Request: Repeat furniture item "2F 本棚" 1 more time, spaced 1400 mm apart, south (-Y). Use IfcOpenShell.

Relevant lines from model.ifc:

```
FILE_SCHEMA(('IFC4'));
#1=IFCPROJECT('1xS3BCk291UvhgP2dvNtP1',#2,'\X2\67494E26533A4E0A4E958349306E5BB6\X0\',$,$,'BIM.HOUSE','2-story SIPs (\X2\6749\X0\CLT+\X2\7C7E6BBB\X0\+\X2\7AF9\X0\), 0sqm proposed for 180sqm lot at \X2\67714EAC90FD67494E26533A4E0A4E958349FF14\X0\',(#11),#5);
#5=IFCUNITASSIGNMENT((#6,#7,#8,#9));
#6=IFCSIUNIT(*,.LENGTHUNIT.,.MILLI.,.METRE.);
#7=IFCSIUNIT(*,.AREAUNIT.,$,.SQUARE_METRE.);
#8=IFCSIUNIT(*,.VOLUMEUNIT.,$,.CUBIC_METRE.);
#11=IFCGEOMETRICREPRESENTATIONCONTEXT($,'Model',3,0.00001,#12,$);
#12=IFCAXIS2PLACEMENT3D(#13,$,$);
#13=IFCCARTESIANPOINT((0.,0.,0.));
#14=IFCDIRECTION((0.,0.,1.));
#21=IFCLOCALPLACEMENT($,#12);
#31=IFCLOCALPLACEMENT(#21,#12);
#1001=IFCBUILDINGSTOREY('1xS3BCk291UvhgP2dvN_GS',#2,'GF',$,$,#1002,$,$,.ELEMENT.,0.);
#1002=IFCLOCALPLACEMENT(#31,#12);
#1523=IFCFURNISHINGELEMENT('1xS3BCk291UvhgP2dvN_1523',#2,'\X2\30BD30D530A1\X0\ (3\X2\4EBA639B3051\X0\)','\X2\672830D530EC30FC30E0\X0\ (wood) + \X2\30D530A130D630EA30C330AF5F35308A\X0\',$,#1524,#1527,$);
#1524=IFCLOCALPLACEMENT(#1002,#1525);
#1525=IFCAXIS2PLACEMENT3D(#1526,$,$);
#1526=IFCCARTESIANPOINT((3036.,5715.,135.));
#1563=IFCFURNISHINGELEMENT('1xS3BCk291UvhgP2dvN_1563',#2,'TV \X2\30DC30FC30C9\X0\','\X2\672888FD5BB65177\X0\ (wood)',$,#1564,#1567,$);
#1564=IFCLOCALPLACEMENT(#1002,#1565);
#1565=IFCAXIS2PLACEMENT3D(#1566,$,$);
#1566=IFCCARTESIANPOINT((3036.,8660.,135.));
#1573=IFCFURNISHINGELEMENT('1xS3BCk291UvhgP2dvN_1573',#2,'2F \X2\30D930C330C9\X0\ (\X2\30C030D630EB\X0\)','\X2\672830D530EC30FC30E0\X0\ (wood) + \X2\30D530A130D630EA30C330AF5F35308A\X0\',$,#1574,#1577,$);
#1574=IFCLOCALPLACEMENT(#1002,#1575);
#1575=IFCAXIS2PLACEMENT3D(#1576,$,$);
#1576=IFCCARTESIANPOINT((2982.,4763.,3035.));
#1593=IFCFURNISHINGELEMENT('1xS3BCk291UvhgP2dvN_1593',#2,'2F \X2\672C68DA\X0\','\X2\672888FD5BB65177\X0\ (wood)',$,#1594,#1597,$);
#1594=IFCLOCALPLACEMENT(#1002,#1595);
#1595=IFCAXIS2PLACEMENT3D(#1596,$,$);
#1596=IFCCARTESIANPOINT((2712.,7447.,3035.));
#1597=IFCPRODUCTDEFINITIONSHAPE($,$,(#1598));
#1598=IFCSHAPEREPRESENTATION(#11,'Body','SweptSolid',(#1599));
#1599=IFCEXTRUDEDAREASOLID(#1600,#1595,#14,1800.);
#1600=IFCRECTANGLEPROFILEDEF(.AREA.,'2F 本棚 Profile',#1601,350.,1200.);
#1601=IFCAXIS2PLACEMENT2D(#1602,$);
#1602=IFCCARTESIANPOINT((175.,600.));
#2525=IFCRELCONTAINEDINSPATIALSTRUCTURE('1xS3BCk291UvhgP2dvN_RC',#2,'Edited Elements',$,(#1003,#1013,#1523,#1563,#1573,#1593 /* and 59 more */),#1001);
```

```python
import numpy as np
import ifcopenshell
import ifcopenshell.api.geometry
import ifcopenshell.api.root
import ifcopenshell.util.element
import ifcopenshell.util.placement

model = ifcopenshell.open("model.ifc")


def reuse_history(source, copy):
    """copy_class also copies each property set's owner history, people and application; keep the originals."""
    for rel in copy.IsDefinedBy:
        if rel.is_a("IfcRelDefinesByProperties") and (history := rel.RelatingPropertyDefinition.OwnerHistory):
            rel.RelatingPropertyDefinition.OwnerHistory = source.OwnerHistory
            ifcopenshell.util.element.remove_deep2(model, history)


source = model.by_guid("1xS3BCk291UvhgP2dvN_1593")
base = ifcopenshell.util.placement.get_local_placement(source.ObjectPlacement)
step = np.array([0.0, -1.0, 0.0]) * 1400.0

for i in range(1, 2):
    copy = ifcopenshell.api.root.copy_class(model, product=source)
    copy.Representation = ifcopenshell.util.element.copy_deep(
        model, source.Representation, exclude=["IfcGeometricRepresentationContext", "IfcRepresentationMap"]
    )
    reuse_history(source, copy)
    matrix = base.copy()
    matrix[:3, 3] += i * step
    print("added at", matrix[:3, 3].round(3) + 0.0)
    ifcopenshell.api.geometry.edit_object_placement(model, product=copy, matrix=matrix, is_si=False)

model.write("model_updated.ifc")
```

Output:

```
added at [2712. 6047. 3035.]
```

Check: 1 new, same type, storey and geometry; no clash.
